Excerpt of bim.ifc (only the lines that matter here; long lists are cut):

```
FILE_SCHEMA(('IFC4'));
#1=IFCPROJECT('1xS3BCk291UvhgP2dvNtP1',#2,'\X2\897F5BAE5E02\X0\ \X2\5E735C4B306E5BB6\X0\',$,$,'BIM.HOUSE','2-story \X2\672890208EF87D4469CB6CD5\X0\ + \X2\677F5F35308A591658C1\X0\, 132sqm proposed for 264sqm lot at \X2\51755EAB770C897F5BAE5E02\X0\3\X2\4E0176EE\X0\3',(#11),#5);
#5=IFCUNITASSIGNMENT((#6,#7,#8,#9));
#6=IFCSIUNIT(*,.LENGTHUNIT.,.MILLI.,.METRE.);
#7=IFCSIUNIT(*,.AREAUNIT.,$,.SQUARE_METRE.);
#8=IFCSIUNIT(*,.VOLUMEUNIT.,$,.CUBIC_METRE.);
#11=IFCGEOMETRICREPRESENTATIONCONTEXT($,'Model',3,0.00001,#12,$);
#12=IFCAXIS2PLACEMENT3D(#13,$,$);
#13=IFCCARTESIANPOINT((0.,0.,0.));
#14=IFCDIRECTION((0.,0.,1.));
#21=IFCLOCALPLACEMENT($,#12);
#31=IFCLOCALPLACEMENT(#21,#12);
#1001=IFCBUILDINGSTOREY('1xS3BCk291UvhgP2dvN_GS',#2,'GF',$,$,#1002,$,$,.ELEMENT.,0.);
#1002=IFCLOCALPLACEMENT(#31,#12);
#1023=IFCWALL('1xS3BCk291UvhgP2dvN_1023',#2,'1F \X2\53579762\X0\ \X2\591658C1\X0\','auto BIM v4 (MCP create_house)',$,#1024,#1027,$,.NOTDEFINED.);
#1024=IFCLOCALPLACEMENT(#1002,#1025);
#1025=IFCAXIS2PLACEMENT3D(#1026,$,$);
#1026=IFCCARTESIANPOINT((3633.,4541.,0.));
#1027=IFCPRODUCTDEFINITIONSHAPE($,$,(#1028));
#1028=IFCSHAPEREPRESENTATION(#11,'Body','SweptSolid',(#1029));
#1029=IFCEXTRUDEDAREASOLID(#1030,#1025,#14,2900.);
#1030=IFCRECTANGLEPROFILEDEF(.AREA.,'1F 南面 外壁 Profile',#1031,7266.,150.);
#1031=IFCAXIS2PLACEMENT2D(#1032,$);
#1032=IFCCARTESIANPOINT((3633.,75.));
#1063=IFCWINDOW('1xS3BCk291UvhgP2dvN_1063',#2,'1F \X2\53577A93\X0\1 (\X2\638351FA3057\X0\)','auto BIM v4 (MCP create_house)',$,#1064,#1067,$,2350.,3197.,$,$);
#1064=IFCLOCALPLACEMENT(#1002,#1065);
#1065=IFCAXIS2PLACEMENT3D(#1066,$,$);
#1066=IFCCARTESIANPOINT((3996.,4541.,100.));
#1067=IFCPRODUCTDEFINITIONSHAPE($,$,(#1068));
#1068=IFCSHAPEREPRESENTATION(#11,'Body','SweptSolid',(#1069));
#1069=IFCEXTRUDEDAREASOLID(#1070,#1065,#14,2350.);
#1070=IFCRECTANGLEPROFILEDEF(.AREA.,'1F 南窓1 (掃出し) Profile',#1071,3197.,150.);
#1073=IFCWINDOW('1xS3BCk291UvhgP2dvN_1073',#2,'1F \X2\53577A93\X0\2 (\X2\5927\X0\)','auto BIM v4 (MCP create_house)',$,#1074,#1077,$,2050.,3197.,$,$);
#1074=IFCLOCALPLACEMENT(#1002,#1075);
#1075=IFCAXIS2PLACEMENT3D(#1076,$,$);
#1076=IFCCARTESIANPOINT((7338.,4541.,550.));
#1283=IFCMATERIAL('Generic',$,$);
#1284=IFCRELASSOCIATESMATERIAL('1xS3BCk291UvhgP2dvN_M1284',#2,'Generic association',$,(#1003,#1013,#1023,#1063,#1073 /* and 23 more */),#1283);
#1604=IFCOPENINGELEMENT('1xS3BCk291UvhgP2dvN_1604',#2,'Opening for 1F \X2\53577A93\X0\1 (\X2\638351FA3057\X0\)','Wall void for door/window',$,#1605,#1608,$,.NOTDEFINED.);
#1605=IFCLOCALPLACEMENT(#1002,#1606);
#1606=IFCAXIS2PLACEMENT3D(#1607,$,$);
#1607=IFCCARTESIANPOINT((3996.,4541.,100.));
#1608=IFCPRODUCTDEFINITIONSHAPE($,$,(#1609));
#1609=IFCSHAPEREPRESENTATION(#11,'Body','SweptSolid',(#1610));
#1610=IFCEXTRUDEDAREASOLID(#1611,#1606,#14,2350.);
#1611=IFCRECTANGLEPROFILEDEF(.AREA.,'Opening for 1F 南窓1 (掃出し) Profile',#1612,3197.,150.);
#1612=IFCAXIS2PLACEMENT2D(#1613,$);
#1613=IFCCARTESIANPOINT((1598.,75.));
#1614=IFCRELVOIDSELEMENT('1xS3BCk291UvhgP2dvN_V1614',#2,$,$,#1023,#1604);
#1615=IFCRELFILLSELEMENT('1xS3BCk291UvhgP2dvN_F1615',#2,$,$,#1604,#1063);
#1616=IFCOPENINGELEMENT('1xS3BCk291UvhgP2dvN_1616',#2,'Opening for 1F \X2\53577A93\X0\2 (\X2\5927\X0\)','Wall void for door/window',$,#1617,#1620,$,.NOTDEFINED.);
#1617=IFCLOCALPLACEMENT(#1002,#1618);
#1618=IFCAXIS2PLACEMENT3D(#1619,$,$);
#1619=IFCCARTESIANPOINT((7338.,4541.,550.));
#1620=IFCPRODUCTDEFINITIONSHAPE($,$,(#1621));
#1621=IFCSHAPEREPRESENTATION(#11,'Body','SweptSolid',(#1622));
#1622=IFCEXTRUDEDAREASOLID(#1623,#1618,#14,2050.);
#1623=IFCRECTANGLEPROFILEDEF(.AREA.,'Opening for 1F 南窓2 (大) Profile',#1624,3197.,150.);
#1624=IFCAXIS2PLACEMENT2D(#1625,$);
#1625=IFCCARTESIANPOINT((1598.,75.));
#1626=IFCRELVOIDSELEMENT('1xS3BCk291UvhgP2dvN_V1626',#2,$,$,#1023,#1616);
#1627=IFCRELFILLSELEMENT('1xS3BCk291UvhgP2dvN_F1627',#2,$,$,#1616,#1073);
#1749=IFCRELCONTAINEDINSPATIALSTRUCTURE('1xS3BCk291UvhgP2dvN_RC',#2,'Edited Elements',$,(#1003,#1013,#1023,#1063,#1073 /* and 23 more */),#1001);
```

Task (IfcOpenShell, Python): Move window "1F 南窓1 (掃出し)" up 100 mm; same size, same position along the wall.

```python
import numpy as np
import ifcopenshell
import ifcopenshell.api.geometry
import ifcopenshell.util.placement
import ifcopenshell.util.unit

model = ifcopenshell.open("bim.ifc")
unit_scale = ifcopenshell.util.unit.calculate_unit_scale(model)

window = model.by_guid("1xS3BCk291UvhgP2dvN_1063")
opening = window.FillsVoids[0].RelatingOpeningElement
dz = 0.1 / unit_scale

shift = np.array([0.0, 0.0, dz])
# The window is not placed relative to its opening, so move both.
for product in (opening, window):
    matrix = ifcopenshell.util.placement.get_local_placement(product.ObjectPlacement)
    matrix[:3, 3] += shift
    ifcopenshell.api.geometry.edit_object_placement(model, product=product, matrix=matrix, is_si=False)

print(f"moved by {dz * unit_scale:+.3f} m")

model.write("bim_edited.ifc")
```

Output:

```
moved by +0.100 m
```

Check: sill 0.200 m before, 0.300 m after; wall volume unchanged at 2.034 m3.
